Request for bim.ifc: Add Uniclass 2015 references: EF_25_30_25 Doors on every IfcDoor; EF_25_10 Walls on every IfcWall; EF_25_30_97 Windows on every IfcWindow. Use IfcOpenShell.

First a look at what the model holds.

```python
import ifcopenshell

model = ifcopenshell.open("bim.ifc")
print(model.schema)
print("classifications:", [c.Name for c in model.by_type("IfcClassification")])
for ifc_class in ("IfcDoor", "IfcRoof", "IfcStair", "IfcWall", "IfcWindow"):
    print(ifc_class, len(model.by_type(ifc_class)))
```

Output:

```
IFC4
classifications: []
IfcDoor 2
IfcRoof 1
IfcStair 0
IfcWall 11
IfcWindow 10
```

```python
import ifcopenshell
import ifcopenshell.api.classification

model = ifcopenshell.open("bim.ifc")

system = ifcopenshell.api.classification.add_classification(model, classification="Uniclass 2015")

codes = {
    "IfcDoor": ("EF_25_30_25", "Doors"),
    "IfcWall": ("EF_25_10", "Walls"),
    "IfcWindow": ("EF_25_30_97", "Windows"),
}
for ifc_class, (code, name) in codes.items():
    products = model.by_type(ifc_class)
    ifcopenshell.api.classification.add_reference(
        model, products=products, classification=system, identification=code, name=name
    )
    print(code, len(products))

model.write("bim_v2.ifc")
```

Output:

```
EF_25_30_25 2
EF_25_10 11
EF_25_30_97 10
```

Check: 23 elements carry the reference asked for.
